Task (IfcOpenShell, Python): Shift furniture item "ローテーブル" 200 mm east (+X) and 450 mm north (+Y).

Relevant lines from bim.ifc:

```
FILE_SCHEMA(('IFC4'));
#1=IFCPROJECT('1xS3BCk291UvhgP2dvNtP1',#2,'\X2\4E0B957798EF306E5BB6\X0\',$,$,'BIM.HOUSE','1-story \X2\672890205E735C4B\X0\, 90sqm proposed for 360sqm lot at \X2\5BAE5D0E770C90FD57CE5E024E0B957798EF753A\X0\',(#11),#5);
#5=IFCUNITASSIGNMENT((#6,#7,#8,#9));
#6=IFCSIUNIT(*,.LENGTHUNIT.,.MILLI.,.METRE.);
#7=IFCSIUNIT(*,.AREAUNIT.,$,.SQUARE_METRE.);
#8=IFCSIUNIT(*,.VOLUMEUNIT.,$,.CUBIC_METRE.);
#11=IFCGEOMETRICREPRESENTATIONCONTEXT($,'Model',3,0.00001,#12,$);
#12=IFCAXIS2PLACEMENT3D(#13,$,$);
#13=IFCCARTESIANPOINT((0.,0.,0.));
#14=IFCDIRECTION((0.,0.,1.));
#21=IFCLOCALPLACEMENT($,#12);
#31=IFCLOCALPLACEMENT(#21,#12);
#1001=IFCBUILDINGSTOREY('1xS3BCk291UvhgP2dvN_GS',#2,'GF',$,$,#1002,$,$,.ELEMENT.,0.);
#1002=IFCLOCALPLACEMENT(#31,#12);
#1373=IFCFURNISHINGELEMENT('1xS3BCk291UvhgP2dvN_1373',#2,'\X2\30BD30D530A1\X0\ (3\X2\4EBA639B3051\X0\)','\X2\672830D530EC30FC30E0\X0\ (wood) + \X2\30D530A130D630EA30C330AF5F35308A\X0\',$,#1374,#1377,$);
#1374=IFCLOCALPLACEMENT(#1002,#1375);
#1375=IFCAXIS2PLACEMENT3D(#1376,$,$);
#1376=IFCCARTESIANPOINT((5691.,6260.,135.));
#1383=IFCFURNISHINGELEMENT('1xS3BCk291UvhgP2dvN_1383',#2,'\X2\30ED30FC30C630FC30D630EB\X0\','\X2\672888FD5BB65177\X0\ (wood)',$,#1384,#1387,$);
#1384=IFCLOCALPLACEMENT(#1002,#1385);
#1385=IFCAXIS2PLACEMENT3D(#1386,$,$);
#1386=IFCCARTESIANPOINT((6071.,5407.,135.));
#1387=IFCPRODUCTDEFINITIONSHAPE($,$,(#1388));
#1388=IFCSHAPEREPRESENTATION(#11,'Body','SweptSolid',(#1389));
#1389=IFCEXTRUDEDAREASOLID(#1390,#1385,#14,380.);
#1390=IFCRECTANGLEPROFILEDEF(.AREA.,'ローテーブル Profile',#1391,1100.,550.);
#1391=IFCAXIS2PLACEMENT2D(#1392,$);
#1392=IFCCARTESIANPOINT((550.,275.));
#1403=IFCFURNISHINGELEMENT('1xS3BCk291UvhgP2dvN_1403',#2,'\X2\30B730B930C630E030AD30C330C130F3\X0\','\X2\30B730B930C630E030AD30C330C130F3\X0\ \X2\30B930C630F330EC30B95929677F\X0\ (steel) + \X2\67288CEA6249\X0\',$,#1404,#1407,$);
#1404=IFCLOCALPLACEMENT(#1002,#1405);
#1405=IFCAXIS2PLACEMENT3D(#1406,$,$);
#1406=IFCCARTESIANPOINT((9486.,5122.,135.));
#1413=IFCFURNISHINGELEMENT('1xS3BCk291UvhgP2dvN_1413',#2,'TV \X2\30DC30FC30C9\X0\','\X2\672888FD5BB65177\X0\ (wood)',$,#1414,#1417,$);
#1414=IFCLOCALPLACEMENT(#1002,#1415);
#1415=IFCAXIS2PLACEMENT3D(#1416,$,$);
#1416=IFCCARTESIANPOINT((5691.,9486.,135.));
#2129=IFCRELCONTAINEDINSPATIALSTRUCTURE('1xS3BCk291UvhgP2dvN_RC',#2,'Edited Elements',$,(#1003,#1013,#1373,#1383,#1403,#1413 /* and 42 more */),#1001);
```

```python
import ifcopenshell
import ifcopenshell.api.geometry
import ifcopenshell.util.placement

model = ifcopenshell.open("bim.ifc")

item = model.by_guid("1xS3BCk291UvhgP2dvN_1383")
matrix = ifcopenshell.util.placement.get_local_placement(item.ObjectPlacement)
matrix[0, 3] += 200.0
matrix[1, 3] += 450.0
ifcopenshell.api.geometry.edit_object_placement(model, product=item, matrix=matrix, is_si=False)

print(ifcopenshell.util.placement.get_local_placement(item.ObjectPlacement).round(3) + 0.0)

model.write("bim_v2.ifc")
```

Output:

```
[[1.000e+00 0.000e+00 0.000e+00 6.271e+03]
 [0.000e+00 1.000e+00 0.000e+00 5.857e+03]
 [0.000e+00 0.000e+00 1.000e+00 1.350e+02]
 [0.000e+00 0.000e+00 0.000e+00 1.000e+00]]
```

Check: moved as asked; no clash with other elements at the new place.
